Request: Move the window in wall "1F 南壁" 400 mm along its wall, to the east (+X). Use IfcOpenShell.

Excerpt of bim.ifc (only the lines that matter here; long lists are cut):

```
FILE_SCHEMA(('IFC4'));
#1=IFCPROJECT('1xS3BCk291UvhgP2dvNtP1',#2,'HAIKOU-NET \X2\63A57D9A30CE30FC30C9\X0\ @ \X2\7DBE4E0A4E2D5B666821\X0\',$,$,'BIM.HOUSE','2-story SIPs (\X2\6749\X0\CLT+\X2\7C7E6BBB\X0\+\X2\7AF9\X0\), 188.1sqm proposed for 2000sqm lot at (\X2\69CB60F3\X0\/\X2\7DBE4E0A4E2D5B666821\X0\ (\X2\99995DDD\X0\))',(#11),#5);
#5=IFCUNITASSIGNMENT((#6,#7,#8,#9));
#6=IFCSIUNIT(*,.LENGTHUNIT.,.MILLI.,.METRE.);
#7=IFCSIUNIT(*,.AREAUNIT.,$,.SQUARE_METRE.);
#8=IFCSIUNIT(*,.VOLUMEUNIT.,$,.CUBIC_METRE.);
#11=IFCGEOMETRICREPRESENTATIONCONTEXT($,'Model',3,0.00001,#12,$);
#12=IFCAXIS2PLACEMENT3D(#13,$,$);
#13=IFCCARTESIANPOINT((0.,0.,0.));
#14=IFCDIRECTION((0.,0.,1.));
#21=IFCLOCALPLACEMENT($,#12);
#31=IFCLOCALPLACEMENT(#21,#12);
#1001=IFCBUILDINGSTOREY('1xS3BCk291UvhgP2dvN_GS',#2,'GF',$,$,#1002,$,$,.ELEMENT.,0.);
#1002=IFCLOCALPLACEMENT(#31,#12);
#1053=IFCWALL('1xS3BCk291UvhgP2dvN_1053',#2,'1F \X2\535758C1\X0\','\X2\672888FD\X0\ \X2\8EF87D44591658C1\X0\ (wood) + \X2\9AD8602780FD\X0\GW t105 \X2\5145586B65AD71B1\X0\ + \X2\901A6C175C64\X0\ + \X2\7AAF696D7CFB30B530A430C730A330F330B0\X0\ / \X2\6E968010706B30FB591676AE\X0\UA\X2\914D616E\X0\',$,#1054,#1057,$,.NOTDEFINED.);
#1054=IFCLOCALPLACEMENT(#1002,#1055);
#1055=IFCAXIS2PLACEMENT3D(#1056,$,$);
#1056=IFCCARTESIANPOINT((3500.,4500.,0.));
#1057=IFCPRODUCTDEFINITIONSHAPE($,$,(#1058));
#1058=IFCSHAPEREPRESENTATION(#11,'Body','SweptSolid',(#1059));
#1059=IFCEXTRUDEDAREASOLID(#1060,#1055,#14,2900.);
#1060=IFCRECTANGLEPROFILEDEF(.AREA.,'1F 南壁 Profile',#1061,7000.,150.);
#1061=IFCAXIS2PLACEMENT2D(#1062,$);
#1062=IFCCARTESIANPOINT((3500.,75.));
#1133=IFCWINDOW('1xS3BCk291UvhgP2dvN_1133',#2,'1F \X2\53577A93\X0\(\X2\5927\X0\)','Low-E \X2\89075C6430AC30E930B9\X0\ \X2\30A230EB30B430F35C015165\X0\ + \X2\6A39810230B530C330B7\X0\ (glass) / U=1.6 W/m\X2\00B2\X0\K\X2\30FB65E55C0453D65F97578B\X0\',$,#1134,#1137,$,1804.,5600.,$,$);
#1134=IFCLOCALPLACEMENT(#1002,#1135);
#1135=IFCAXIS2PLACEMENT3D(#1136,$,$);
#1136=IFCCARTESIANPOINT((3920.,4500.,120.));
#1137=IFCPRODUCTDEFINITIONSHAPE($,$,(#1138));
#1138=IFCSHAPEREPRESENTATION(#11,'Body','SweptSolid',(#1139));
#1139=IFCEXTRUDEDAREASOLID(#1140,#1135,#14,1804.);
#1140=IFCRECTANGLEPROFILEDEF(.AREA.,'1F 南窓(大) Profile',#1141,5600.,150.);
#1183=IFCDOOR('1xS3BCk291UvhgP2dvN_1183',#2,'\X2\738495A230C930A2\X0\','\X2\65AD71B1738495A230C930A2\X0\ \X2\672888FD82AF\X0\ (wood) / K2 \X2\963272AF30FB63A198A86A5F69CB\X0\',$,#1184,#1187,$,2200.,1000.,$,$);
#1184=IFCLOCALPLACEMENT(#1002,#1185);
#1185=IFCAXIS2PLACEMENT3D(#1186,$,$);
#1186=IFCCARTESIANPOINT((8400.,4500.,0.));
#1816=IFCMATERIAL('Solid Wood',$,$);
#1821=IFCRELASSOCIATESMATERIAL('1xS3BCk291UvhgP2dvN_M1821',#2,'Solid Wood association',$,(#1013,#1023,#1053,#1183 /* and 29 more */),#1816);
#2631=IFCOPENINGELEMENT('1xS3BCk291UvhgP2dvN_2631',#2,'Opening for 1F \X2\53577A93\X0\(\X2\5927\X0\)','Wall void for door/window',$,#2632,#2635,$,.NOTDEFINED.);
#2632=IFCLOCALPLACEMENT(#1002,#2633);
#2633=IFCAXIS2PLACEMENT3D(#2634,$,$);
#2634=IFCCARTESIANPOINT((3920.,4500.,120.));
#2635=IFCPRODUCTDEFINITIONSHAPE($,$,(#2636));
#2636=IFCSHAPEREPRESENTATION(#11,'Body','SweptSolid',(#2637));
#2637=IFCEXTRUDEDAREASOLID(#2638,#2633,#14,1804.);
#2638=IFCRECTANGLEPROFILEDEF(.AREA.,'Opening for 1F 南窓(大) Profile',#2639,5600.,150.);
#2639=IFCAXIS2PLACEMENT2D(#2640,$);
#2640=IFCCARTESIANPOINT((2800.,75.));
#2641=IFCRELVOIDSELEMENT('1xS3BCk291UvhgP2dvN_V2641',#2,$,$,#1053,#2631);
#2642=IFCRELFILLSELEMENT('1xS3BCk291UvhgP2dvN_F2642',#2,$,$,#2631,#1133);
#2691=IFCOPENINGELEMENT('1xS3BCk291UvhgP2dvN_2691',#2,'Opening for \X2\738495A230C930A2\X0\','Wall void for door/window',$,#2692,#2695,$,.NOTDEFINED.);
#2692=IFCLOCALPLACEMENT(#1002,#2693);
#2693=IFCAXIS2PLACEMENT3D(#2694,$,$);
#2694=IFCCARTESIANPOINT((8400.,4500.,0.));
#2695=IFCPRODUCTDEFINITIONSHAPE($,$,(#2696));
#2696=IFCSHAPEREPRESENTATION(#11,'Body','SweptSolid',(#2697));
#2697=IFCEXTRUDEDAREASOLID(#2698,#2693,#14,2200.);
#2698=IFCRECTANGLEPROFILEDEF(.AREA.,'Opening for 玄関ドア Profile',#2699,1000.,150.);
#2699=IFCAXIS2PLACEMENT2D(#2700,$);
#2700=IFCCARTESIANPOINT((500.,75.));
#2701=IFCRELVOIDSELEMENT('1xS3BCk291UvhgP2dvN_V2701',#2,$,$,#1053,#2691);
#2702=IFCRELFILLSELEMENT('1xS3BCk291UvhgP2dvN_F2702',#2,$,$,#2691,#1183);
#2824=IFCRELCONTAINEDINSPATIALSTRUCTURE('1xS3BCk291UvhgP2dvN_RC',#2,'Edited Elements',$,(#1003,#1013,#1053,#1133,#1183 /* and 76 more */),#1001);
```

```python
import ifcopenshell
import ifcopenshell.api.geometry
import ifcopenshell.util.placement

model = ifcopenshell.open("bim.ifc")

window = model.by_guid("1xS3BCk291UvhgP2dvN_1133")
opening = window.FillsVoids[0].RelatingOpeningElement
wall = opening.VoidsElements[0].RelatingBuildingElement

wall_matrix = ifcopenshell.util.placement.get_local_placement(wall.ObjectPlacement)
shift = wall_matrix[:3, 0] * 400.0
before = ifcopenshell.util.placement.get_local_placement(window.ObjectPlacement)[:3, 3].copy()

# The window is not placed relative to its opening, so move both.
for product in (opening, window):
    matrix = ifcopenshell.util.placement.get_local_placement(product.ObjectPlacement)
    matrix[:3, 3] += shift
    ifcopenshell.api.geometry.edit_object_placement(model, product=product, matrix=matrix, is_si=False)

after = ifcopenshell.util.placement.get_local_placement(window.ObjectPlacement)[:3, 3]
print("window moved by", (after - before).round(3) + 0.0)

model.write("bim_updated.ifc")
```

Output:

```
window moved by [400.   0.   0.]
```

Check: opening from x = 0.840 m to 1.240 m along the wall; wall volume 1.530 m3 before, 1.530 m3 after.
